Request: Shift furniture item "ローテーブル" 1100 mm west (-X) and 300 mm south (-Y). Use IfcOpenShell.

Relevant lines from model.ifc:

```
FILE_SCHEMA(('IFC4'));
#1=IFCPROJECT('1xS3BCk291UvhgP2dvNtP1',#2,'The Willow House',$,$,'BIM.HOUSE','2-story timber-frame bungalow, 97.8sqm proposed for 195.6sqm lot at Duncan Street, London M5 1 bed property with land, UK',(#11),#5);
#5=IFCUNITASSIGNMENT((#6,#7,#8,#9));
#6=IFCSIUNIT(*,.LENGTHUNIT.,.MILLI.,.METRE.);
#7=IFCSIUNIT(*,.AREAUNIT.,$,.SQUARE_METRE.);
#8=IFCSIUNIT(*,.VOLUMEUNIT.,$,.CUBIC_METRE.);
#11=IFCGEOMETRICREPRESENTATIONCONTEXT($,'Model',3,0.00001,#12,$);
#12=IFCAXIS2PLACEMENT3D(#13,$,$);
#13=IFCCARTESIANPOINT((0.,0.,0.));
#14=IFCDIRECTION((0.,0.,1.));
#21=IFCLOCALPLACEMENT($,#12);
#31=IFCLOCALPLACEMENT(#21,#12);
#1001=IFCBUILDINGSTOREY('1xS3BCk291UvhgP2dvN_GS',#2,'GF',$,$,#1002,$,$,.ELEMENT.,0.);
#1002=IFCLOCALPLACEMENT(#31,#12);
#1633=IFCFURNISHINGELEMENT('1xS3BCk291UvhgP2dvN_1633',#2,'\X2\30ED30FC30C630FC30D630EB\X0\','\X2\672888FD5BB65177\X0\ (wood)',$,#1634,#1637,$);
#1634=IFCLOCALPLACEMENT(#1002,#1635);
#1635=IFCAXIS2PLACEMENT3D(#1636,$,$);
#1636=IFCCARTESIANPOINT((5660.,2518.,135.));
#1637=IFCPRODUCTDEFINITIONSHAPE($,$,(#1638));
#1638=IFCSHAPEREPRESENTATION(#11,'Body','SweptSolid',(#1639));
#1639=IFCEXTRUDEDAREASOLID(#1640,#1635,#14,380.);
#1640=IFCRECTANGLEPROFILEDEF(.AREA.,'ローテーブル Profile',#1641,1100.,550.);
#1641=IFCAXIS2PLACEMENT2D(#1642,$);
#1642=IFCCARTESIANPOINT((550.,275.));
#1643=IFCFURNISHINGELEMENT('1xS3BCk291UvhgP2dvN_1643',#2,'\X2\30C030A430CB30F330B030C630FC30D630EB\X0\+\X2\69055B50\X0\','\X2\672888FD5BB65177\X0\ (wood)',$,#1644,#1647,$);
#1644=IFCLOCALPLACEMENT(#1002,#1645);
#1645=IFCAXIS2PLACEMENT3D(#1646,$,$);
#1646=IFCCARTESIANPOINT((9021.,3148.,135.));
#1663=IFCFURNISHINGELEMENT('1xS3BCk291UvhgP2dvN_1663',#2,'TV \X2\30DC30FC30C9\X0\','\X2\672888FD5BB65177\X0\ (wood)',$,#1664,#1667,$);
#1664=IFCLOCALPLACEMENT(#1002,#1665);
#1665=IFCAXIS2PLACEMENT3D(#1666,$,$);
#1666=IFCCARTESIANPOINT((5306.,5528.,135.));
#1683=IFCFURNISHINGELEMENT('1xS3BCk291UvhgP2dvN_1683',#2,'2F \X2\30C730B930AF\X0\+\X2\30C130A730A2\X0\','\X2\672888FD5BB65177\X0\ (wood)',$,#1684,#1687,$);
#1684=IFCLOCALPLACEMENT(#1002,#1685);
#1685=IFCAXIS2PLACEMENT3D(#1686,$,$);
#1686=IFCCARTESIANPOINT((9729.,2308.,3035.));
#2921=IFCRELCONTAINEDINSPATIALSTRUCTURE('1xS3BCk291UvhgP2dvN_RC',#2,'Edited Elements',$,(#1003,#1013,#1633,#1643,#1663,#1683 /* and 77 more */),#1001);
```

```python
import ifcopenshell
import ifcopenshell.api.geometry
import ifcopenshell.util.placement

model = ifcopenshell.open("model.ifc")

item = model.by_guid("1xS3BCk291UvhgP2dvN_1633")
matrix = ifcopenshell.util.placement.get_local_placement(item.ObjectPlacement)
matrix[0, 3] -= 1100.0
matrix[1, 3] -= 300.0
ifcopenshell.api.geometry.edit_object_placement(model, product=item, matrix=matrix, is_si=False)

print(ifcopenshell.util.placement.get_local_placement(item.ObjectPlacement).round(3) + 0.0)

model.write("model-out.ifc")
```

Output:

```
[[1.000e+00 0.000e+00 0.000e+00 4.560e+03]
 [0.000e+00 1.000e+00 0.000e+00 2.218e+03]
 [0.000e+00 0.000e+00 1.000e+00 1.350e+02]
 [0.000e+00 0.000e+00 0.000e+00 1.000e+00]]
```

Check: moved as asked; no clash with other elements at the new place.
